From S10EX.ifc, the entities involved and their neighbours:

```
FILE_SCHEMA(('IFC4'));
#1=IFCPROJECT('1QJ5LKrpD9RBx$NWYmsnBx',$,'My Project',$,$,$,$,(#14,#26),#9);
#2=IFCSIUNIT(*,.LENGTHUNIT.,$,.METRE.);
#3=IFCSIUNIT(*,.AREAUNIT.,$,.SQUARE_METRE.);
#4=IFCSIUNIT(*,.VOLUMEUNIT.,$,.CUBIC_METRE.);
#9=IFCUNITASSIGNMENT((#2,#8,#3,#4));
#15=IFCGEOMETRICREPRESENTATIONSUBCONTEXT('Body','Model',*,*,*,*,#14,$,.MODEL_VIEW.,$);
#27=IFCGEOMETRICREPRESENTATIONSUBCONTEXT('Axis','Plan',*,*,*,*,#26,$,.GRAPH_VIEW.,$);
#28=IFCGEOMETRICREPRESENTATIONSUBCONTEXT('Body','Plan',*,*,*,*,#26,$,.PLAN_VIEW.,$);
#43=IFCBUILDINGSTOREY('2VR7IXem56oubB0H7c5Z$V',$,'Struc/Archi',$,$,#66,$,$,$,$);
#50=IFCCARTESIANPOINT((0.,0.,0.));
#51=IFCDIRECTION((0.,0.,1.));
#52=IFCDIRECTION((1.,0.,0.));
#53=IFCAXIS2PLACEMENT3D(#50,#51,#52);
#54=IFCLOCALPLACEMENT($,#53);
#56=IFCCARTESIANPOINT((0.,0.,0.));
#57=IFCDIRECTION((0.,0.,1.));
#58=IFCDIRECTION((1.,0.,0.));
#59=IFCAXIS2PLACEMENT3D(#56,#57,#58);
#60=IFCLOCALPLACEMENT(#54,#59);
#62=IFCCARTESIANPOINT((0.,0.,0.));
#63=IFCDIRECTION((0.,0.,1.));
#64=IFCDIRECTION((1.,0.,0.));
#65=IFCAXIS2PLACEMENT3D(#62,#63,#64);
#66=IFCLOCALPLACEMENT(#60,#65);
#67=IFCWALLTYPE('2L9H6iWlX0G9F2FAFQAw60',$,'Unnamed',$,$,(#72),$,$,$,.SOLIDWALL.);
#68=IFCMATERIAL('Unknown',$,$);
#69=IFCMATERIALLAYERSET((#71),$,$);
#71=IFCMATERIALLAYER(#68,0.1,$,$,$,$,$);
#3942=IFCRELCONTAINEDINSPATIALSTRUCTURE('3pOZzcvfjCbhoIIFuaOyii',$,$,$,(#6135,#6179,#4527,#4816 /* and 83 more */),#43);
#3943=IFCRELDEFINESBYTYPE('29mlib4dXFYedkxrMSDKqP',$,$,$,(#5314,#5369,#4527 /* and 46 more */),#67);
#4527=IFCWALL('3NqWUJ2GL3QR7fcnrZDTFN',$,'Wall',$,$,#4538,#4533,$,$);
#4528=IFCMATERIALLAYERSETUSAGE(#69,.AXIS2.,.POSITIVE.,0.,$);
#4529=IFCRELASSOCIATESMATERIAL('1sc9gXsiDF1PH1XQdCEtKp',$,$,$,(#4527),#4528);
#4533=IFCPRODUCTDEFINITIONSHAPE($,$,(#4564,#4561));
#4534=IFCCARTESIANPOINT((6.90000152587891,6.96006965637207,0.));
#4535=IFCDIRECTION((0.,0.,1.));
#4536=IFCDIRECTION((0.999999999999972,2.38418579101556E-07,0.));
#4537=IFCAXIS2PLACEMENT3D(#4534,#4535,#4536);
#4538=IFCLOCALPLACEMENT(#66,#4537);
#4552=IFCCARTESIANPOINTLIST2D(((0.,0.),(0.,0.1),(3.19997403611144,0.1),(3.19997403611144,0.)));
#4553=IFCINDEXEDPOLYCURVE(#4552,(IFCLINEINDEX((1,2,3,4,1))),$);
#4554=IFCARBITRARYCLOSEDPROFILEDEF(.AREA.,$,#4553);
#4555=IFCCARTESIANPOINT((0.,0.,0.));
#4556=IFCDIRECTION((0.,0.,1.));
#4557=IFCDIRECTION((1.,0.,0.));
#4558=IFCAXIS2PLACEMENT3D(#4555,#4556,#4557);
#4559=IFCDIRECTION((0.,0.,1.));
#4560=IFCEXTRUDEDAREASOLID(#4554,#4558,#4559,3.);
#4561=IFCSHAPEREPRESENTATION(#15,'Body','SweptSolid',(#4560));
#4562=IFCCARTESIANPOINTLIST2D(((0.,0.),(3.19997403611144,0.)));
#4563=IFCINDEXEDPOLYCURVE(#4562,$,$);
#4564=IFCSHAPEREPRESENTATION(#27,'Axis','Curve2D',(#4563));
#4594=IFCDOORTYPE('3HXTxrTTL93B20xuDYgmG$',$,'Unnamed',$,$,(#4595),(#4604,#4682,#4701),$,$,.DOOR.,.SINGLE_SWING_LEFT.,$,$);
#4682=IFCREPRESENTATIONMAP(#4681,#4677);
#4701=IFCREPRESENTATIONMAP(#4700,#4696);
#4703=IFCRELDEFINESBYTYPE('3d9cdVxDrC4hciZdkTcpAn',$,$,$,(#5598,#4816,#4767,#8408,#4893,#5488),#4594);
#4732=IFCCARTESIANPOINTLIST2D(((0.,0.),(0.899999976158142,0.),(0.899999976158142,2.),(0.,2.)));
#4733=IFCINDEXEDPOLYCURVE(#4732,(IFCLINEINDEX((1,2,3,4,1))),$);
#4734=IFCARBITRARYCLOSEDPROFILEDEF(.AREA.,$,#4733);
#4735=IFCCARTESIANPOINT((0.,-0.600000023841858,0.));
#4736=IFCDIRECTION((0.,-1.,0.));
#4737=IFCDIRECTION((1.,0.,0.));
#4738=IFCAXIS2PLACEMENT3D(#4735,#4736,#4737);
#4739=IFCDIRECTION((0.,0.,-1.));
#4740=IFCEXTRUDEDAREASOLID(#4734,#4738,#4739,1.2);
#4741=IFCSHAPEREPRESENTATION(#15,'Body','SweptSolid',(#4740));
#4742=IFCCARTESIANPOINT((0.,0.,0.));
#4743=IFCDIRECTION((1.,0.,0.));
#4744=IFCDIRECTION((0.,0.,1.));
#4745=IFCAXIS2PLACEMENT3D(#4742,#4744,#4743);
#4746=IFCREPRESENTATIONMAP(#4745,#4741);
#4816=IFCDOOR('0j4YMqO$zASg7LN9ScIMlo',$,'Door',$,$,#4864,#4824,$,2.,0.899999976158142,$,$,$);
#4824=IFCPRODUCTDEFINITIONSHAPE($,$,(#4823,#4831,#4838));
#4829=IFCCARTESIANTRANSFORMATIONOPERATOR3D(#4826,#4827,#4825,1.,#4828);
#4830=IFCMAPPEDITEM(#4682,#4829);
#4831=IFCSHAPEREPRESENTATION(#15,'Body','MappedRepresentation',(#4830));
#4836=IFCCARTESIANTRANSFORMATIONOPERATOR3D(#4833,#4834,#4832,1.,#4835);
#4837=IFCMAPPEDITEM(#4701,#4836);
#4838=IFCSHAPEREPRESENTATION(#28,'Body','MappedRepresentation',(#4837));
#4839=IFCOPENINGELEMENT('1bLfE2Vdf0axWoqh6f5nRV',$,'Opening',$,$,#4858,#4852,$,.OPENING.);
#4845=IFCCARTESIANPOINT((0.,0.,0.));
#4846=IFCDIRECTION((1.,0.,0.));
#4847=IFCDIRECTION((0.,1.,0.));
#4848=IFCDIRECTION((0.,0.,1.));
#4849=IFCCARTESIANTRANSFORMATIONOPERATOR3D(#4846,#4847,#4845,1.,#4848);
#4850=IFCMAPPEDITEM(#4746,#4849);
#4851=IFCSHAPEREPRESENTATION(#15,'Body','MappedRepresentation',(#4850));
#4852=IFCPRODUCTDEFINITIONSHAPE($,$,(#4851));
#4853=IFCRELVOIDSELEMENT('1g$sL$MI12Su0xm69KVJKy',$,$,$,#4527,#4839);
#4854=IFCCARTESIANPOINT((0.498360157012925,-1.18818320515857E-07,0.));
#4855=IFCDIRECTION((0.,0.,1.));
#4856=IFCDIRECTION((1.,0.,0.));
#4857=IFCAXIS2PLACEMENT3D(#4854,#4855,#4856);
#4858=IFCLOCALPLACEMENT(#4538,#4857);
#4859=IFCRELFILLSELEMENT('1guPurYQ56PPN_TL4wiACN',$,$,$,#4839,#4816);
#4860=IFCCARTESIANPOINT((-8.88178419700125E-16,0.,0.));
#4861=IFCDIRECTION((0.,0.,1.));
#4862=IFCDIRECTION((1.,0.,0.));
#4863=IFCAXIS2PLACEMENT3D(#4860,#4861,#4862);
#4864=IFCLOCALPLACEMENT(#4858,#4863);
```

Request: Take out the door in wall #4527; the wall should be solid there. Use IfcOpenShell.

```python
import ifcopenshell
import ifcopenshell.api.feature
import ifcopenshell.api.root
import ifcopenshell.geom
import ifcopenshell.util.shape

model = ifcopenshell.open("S10EX.ifc")
settings = ifcopenshell.geom.settings()


def volume(element):
    """Net volume in cubic metres, openings subtracted."""
    shape = ifcopenshell.geom.create_shape(settings, element)
    return ifcopenshell.util.shape.get_volume(shape.geometry)


door = model.by_id(4816)
opening = door.FillsVoids[0].RelatingOpeningElement
wall = opening.VoidsElements[0].RelatingBuildingElement
before = volume(wall)

ifcopenshell.api.root.remove_product(model, product=door)
ifcopenshell.api.feature.remove_feature(model, feature=opening)

after = volume(wall)

print(f"wall volume {before:.3f} -> {after:.3f} m3")

model.write("S10EX_edited.ifc")
```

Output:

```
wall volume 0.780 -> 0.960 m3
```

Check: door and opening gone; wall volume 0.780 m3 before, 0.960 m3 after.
